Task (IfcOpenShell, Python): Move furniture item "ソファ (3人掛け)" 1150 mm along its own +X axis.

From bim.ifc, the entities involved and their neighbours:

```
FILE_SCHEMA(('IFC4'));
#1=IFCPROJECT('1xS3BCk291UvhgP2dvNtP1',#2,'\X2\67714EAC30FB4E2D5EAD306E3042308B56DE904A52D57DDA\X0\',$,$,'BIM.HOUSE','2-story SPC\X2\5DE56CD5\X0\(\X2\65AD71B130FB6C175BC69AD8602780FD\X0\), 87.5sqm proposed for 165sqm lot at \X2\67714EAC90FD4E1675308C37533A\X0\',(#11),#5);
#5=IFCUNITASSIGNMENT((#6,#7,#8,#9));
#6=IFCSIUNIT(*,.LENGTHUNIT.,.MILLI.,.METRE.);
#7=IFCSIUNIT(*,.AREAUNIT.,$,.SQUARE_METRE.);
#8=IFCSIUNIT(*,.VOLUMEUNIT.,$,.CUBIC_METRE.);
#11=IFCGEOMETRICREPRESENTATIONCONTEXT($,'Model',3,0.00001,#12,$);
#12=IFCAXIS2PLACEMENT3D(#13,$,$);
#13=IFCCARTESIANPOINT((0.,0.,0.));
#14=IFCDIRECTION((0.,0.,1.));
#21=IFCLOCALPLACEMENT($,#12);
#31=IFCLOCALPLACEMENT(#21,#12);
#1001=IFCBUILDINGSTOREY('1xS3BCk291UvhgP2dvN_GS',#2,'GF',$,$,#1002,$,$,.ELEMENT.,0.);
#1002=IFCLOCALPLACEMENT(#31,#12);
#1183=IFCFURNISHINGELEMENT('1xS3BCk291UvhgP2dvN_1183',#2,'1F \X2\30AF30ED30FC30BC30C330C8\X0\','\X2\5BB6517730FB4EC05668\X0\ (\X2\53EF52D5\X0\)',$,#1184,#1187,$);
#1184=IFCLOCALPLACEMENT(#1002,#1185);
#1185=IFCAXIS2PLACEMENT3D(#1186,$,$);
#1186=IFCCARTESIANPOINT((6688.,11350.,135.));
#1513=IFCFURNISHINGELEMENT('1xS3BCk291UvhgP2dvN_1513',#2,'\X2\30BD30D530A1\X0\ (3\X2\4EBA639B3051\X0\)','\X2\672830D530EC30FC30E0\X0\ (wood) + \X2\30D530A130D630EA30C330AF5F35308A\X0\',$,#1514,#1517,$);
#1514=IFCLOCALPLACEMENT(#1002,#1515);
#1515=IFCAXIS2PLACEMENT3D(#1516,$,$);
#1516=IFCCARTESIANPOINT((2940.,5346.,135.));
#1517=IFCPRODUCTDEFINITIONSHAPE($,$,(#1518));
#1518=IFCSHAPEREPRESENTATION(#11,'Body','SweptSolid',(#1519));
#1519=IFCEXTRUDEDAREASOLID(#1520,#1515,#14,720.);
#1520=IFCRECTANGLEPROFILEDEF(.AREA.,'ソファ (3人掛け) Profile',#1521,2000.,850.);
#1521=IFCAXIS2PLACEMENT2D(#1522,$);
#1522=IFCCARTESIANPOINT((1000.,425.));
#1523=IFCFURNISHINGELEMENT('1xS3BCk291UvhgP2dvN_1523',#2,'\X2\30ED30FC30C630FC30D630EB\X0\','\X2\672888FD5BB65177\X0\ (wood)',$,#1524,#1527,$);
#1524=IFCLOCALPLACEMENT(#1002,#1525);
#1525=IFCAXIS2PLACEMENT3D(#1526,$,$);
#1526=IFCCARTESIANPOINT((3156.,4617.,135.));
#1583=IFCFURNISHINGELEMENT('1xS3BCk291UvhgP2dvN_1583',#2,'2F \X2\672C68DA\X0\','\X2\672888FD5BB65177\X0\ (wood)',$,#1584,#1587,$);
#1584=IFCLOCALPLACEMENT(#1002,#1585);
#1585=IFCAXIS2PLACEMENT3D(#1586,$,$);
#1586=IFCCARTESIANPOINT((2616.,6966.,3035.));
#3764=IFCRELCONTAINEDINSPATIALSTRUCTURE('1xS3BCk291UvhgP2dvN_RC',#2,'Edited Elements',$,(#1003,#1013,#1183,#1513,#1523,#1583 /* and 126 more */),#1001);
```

```python
import ifcopenshell
import ifcopenshell.api.geometry
import ifcopenshell.util.placement

model = ifcopenshell.open("bim.ifc")

item = model.by_guid("1xS3BCk291UvhgP2dvN_1513")
matrix = ifcopenshell.util.placement.get_local_placement(item.ObjectPlacement)
matrix[:3, 3] += matrix[:3, 0] * 1150.0
ifcopenshell.api.geometry.edit_object_placement(model, product=item, matrix=matrix, is_si=False)

print(ifcopenshell.util.placement.get_local_placement(item.ObjectPlacement).round(3) + 0.0)

model.write("bim_rev.ifc")
```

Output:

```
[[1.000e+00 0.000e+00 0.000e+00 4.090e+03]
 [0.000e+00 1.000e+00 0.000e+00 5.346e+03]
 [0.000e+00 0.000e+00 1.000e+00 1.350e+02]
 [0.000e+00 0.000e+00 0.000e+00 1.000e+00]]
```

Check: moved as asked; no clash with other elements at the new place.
